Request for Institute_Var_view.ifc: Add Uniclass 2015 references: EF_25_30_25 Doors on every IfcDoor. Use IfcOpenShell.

First a look at what the model holds.

```python
import ifcopenshell

model = ifcopenshell.open("Institute_Var_view.ifc")
print(model.schema)
print("classifications:", [c.Name for c in model.by_type("IfcClassification")])
for ifc_class in ("IfcDoor", "IfcRoof", "IfcStair", "IfcWall", "IfcWindow"):
    print(ifc_class, len(model.by_type(ifc_class)))
```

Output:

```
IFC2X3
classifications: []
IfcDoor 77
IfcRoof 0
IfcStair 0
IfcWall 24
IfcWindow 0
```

```python
import ifcopenshell
import ifcopenshell.api.classification

model = ifcopenshell.open("Institute_Var_view.ifc")

# IFC2X3 requires Source and Edition and has no link from the project to the system.
system = model.create_entity("IfcClassification", Source="NBS", Edition="2015", Name="Uniclass 2015")

codes = {
    "IfcDoor": ("EF_25_30_25", "Doors"),
}
for ifc_class, (code, name) in codes.items():
    products = model.by_type(ifc_class)
    ifcopenshell.api.classification.add_reference(
        model, products=products, classification=system, identification=code, name=name
    )
    print(code, len(products))

model.write("Institute_Var_view_rev.ifc")
```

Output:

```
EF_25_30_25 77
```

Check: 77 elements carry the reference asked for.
